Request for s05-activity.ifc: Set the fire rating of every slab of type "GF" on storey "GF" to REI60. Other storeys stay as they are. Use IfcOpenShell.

First a look at what the model holds.

```python
import ifcopenshell
import ifcopenshell.util.element

model = ifcopenshell.open("s05-activity.ifc")
print(model.schema)
storey = next(s for s in model.by_type("IfcBuildingStorey") if s.Name == "GF")
slabs = [e for e in ifcopenshell.util.element.get_decomposition(storey) if e.is_a("IfcSlab")]
seen = {}
for e in slabs:
    element_type = ifcopenshell.util.element.get_type(e)
    key = (element_type.Name if element_type != e and element_type else None, ifcopenshell.util.element.get_pset(e, "Pset_SlabCommon", "FireRating"))
    seen[key] = seen.get(key, 0) + 1
for (name, value), count in sorted(seen.items(), key=str):
    print(count, "x", name, "|", value)
```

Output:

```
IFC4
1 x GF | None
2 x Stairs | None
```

```python
import ifcopenshell
import ifcopenshell.api.pset
import ifcopenshell.util.element

model = ifcopenshell.open("s05-activity.ifc")

storey = next(s for s in model.by_type("IfcBuildingStorey") if s.Name == "GF")
slabs = [e for e in ifcopenshell.util.element.get_decomposition(storey) if e.is_a("IfcSlab")]

count = 0
for e in slabs:
    element_type = ifcopenshell.util.element.get_type(e)
    if element_type in (None, e) or element_type.Name != "GF":
        continue
    # add_pset returns the element's existing set when there is one.
    pset = ifcopenshell.api.pset.add_pset(model, product=e, name="Pset_SlabCommon")
    ifcopenshell.api.pset.edit_pset(model, pset=pset, properties={"FireRating": "REI60"})
    count += 1

print(count, "slabs updated")

model.write("s05-activity-out.ifc")
```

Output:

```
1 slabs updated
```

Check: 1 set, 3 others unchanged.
